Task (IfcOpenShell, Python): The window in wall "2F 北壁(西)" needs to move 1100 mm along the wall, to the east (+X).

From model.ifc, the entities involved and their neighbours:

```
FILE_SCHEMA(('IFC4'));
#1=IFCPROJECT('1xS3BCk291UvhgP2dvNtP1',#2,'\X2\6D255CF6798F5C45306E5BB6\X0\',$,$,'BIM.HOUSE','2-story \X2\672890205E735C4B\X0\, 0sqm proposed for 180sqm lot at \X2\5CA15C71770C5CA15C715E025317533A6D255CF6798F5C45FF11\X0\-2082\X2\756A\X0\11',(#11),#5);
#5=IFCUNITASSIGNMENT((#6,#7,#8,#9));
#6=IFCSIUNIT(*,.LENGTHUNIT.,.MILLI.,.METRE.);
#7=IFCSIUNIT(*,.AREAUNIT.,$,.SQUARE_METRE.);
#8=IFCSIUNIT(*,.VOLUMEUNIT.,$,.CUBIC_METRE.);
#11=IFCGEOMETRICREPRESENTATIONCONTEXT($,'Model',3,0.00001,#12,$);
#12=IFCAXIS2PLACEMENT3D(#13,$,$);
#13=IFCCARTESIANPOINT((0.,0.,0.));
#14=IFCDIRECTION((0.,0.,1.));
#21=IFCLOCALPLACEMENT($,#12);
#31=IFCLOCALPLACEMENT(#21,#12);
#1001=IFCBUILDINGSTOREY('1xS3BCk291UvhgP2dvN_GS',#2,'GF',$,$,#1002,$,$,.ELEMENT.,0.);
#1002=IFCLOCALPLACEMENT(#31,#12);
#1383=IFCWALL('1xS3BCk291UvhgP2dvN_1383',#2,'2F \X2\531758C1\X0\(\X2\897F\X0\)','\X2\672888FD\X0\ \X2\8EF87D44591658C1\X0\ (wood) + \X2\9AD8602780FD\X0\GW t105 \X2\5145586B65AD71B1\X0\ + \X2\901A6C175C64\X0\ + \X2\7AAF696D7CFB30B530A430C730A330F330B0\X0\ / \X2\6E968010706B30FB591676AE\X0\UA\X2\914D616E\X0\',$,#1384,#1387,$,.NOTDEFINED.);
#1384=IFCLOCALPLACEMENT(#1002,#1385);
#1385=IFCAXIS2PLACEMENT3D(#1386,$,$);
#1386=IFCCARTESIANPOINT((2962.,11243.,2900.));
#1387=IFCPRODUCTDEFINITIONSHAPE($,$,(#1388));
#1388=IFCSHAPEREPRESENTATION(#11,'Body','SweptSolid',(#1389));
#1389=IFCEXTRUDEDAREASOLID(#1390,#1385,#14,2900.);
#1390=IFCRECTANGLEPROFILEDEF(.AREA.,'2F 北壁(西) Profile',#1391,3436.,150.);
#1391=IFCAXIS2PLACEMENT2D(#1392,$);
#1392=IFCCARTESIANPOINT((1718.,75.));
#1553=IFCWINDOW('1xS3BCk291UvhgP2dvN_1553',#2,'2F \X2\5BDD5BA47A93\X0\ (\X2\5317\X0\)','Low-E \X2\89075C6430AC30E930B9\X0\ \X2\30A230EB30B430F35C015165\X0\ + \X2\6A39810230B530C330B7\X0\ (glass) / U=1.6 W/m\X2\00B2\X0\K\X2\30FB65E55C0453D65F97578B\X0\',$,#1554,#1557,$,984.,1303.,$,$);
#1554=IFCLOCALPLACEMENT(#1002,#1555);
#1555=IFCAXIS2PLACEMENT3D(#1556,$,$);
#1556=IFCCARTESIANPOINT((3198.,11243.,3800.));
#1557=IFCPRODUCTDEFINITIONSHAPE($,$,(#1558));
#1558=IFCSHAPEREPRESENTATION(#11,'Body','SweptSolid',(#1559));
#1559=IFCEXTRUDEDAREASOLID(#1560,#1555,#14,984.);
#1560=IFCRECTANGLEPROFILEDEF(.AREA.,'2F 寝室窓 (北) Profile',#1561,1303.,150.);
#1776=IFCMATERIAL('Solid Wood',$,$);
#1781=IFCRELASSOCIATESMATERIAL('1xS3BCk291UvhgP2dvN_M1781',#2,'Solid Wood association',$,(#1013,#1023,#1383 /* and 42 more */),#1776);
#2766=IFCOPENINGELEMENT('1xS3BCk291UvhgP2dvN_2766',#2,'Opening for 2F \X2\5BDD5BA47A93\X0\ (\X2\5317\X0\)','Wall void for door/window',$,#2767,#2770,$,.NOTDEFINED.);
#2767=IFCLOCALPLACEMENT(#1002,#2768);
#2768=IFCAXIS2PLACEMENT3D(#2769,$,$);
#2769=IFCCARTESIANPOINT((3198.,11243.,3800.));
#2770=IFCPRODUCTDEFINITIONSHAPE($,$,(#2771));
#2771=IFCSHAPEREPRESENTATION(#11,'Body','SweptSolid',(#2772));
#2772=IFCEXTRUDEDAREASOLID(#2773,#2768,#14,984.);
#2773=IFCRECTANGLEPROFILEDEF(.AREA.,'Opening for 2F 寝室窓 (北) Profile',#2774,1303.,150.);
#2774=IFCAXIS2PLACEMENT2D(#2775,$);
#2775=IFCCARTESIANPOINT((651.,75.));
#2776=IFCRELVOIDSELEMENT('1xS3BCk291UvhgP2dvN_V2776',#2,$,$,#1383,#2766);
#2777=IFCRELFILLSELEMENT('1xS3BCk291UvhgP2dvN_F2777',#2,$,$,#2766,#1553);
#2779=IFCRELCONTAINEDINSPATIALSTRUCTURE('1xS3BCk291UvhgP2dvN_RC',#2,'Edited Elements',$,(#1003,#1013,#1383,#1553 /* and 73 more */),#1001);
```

```python
import ifcopenshell
import ifcopenshell.api.geometry
import ifcopenshell.util.placement
import ifcopenshell.util.unit

model = ifcopenshell.open("model.ifc")
unit_scale = ifcopenshell.util.unit.calculate_unit_scale(model)

window = model.by_id(1553)
opening = window.FillsVoids[0].RelatingOpeningElement
wall = opening.VoidsElements[0].RelatingBuildingElement

wall_matrix = ifcopenshell.util.placement.get_local_placement(wall.ObjectPlacement)
shift = wall_matrix[:3, 0] * 1.1 / unit_scale
before = ifcopenshell.util.placement.get_local_placement(window.ObjectPlacement)[:3, 3].copy()

# The window is not placed relative to its opening, so move both.
for product in (opening, window):
    matrix = ifcopenshell.util.placement.get_local_placement(product.ObjectPlacement)
    matrix[:3, 3] += shift
    ifcopenshell.api.geometry.edit_object_placement(model, product=product, matrix=matrix, is_si=False)

after = ifcopenshell.util.placement.get_local_placement(window.ObjectPlacement)[:3, 3]
print("window moved by", (after - before).round(3) + 0.0)

model.write("model_v2.ifc")
```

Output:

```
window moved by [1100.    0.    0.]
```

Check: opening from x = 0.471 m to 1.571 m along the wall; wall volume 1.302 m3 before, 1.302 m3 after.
